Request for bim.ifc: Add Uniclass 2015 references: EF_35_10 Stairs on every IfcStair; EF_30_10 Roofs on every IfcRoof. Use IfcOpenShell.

First a look at what the model holds.

```python
import ifcopenshell

model = ifcopenshell.open("bim.ifc")
print(model.schema)
print("classifications:", [c.Name for c in model.by_type("IfcClassification")])
for ifc_class in ("IfcDoor", "IfcRoof", "IfcStair", "IfcWall", "IfcWindow"):
    print(ifc_class, len(model.by_type(ifc_class)))
```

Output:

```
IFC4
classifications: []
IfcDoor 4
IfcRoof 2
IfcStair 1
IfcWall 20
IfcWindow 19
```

```python
import ifcopenshell
import ifcopenshell.api.classification

model = ifcopenshell.open("bim.ifc")

system = ifcopenshell.api.classification.add_classification(model, classification="Uniclass 2015")

codes = {
    "IfcStair": ("EF_35_10", "Stairs"),
    "IfcRoof": ("EF_30_10", "Roofs"),
}
for ifc_class, (code, name) in codes.items():
    products = model.by_type(ifc_class)
    ifcopenshell.api.classification.add_reference(
        model, products=products, classification=system, identification=code, name=name
    )
    print(code, len(products))

model.write("bim_updated.ifc")
```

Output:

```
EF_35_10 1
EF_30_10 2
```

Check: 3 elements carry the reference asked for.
